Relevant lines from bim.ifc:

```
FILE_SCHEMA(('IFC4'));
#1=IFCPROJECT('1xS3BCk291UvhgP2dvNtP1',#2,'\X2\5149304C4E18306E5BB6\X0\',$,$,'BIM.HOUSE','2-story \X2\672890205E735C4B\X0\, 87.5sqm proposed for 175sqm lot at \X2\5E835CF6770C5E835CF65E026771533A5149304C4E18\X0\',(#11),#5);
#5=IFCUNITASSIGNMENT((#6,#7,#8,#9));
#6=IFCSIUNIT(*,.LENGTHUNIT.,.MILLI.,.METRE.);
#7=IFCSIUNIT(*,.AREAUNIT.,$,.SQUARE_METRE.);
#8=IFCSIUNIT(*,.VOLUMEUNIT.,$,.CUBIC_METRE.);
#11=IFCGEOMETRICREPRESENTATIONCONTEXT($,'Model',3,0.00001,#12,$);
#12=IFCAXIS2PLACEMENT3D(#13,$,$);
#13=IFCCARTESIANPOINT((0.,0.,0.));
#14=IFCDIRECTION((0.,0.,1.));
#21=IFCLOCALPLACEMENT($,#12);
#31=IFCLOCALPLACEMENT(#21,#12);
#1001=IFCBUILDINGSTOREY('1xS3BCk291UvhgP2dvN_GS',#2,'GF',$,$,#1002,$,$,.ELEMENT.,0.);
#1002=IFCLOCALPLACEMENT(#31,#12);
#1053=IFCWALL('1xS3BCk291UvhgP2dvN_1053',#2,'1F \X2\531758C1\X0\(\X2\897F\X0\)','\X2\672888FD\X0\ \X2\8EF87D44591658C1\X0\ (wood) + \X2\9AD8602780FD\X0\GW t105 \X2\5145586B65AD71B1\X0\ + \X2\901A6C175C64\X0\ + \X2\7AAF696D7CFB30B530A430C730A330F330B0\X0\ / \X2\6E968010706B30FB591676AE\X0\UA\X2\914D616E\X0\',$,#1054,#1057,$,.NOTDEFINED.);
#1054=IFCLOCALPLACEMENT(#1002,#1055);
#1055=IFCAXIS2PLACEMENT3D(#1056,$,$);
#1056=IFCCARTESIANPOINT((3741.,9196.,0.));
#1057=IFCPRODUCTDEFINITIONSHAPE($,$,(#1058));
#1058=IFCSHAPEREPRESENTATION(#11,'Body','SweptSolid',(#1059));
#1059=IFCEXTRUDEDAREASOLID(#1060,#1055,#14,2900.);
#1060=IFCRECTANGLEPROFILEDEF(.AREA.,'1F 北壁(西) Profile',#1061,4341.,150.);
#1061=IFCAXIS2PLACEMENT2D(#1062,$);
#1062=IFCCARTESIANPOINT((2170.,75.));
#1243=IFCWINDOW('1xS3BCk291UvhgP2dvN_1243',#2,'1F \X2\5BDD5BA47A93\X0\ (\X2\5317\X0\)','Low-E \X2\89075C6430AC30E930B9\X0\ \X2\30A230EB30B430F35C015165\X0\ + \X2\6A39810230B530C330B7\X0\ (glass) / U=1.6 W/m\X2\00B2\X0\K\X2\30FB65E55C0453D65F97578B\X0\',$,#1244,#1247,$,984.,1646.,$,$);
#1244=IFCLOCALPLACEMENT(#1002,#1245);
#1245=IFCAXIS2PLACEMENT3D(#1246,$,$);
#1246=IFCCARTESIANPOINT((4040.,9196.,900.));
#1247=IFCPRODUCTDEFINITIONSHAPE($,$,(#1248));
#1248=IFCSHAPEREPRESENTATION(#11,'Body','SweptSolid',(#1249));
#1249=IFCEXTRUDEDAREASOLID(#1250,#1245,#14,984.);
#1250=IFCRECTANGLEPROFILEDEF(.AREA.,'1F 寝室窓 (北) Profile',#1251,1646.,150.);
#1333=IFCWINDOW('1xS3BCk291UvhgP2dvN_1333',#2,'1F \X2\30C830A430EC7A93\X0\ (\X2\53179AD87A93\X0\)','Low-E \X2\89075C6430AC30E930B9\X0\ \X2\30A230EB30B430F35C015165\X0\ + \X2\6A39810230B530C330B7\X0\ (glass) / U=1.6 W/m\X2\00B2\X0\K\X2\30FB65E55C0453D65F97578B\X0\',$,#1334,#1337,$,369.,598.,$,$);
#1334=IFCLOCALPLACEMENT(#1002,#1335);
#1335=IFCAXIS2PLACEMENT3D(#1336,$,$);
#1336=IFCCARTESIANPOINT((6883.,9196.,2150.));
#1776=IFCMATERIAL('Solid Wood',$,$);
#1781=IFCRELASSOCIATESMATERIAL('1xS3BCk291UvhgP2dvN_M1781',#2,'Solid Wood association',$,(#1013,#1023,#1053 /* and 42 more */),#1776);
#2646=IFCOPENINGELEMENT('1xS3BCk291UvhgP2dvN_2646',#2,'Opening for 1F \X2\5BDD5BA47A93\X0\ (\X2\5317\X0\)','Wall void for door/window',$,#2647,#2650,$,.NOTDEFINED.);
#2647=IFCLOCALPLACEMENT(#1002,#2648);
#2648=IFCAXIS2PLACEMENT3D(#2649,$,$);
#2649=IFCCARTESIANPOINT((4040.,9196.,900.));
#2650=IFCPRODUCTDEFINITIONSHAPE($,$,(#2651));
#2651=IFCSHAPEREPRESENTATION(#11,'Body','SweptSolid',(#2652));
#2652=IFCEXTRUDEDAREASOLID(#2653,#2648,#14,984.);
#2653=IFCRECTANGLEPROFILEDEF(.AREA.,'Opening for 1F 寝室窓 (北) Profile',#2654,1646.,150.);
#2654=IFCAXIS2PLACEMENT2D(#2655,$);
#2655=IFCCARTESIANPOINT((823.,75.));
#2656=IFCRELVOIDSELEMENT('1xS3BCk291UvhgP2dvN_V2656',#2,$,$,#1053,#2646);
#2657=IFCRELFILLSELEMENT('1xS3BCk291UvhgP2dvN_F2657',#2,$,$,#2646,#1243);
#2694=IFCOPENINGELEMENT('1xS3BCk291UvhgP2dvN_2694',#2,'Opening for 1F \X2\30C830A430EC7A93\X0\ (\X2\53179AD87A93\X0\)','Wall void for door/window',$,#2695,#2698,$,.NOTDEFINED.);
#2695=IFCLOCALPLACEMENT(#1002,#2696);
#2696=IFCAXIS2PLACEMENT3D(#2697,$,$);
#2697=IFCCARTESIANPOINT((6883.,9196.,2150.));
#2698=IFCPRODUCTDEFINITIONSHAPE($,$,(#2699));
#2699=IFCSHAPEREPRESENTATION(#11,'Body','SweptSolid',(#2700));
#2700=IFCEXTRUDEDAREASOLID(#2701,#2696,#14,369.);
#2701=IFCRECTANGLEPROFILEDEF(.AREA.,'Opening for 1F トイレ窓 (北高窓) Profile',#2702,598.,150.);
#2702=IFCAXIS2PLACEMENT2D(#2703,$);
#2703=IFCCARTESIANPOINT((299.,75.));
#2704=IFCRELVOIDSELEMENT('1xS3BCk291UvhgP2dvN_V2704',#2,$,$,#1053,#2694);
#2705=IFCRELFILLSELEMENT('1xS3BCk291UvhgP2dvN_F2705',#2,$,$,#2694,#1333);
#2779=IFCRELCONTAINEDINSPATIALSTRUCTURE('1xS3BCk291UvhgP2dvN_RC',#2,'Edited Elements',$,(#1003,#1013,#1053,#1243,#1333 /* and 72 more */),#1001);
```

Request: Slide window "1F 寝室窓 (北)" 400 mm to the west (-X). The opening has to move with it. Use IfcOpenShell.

```python
import ifcopenshell
import ifcopenshell.api.geometry
import ifcopenshell.util.placement

model = ifcopenshell.open("bim.ifc")

window = model.by_guid("1xS3BCk291UvhgP2dvN_1243")
opening = window.FillsVoids[0].RelatingOpeningElement
wall = opening.VoidsElements[0].RelatingBuildingElement

wall_matrix = ifcopenshell.util.placement.get_local_placement(wall.ObjectPlacement)
shift = wall_matrix[:3, 0] * -400.0
before = ifcopenshell.util.placement.get_local_placement(window.ObjectPlacement)[:3, 3].copy()

# The window is not placed relative to its opening, so move both.
for product in (opening, window):
    matrix = ifcopenshell.util.placement.get_local_placement(product.ObjectPlacement)
    matrix[:3, 3] += shift
    ifcopenshell.api.geometry.edit_object_placement(model, product=product, matrix=matrix, is_si=False)

after = ifcopenshell.util.placement.get_local_placement(window.ObjectPlacement)[:3, 3]
print("window moved by", (after - before).round(3) + 0.0)

model.write("bim_rev.ifc")
```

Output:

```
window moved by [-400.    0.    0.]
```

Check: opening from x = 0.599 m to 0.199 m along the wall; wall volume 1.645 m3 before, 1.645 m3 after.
